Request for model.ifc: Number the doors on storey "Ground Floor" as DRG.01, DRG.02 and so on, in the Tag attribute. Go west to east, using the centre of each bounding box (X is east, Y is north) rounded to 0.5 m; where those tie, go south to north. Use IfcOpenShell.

First a look at what the model holds.

```python
import ifcopenshell
import ifcopenshell.util.element
import ifcopenshell.util.placement

model = ifcopenshell.open("model.ifc")
print(model.schema)
storey = next(s for s in model.by_type("IfcBuildingStorey") if s.Name == "Ground Floor")
doors = [e for e in ifcopenshell.util.element.get_decomposition(storey) if e.is_a("IfcDoor")]
for e in sorted(doors, key=lambda e: e.id()):
    origin = ifcopenshell.util.placement.get_local_placement(e.ObjectPlacement)[:3, 3]
    print(e.id(), e.Tag, e.Name, origin.round(2) + 0.0, sep=" | ")
```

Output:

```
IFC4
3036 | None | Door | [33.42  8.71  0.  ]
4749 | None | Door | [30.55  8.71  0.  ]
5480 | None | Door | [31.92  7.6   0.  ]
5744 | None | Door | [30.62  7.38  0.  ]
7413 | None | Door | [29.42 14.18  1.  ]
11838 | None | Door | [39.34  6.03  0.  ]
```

```python
import ifcopenshell
import ifcopenshell.geom
import ifcopenshell.util.element
import ifcopenshell.util.shape

model = ifcopenshell.open("model.ifc")
settings = ifcopenshell.geom.settings()
settings.set("use-world-coords", True)


def centre(element):
    shape = ifcopenshell.geom.create_shape(settings, element)
    return ifcopenshell.util.shape.get_bbox_centroid(shape.geometry)


storey = next(s for s in model.by_type("IfcBuildingStorey") if s.Name == "Ground Floor")
doors = [e for e in ifcopenshell.util.element.get_decomposition(storey) if e.is_a("IfcDoor")]

# Insertion points can sit at a corner or the storey origin, so sort by the geometry (in metres).
centres = {e: centre(e) for e in doors}
doors.sort(key=lambda e: (round(centres[e][0] / 0.5), centres[e][1]))

for i, e in enumerate(doors, start=1):
    number = f"DRG.{i:02d}"
    e.Tag = number
    print(e.id(), number)

model.write("model_rev.ifc")
```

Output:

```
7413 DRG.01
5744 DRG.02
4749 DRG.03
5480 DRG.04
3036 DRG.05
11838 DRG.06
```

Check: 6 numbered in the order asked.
